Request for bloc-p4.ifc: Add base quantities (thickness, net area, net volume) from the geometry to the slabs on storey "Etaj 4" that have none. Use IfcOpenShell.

First a look at what the model holds.

```python
import ifcopenshell
import ifcopenshell.util.element
import ifcopenshell.util.unit

model = ifcopenshell.open("bloc-p4.ifc")
print(model.schema)
for unit_type in ("LENGTHUNIT", "AREAUNIT", "VOLUMEUNIT"):
    print(unit_type, ifcopenshell.util.unit.calculate_unit_scale(model, unit_type))
storey = next(s for s in model.by_type("IfcBuildingStorey") if s.Name == "Etaj 4")
slabs = [e for e in ifcopenshell.util.element.get_decomposition(storey) if e.is_a("IfcSlab")]
for e in sorted(slabs, key=lambda e: e.id()):
    print(e.id(), e.is_a(), e.Name, list(ifcopenshell.util.element.get_psets(e, qtos_only=True)), sep=" | ")
```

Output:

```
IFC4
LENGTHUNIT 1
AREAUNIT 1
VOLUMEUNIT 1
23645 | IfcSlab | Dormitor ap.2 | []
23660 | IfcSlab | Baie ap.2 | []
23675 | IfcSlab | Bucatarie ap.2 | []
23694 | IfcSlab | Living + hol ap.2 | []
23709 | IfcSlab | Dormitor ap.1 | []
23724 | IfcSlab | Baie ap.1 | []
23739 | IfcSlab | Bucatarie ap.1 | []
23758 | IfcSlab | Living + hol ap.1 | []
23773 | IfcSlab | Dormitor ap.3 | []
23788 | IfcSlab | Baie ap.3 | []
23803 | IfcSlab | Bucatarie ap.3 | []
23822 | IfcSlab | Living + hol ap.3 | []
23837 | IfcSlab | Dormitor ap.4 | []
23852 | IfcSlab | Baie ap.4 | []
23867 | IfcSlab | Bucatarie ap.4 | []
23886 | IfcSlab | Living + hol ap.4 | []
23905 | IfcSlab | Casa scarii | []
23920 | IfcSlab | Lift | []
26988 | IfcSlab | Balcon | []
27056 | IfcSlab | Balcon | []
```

```python
import ifcopenshell
import ifcopenshell.api.pset
import ifcopenshell.geom
import ifcopenshell.util.element
import ifcopenshell.util.shape
import ifcopenshell.util.unit

model = ifcopenshell.open("bloc-p4.ifc")
unit_scale = ifcopenshell.util.unit.calculate_unit_scale(model)
area_scale = ifcopenshell.util.unit.calculate_unit_scale(model, "AREAUNIT")
volume_scale = ifcopenshell.util.unit.calculate_unit_scale(model, "VOLUMEUNIT")
settings = ifcopenshell.geom.settings()

storey = next(s for s in model.by_type("IfcBuildingStorey") if s.Name == "Etaj 4")
slabs = [e for e in ifcopenshell.util.element.get_decomposition(storey) if e.is_a("IfcSlab")]

for e in sorted(slabs, key=lambda e: e.id()):
    if ifcopenshell.util.element.get_psets(e, qtos_only=True, should_inherit=False):
        continue
    # Geometry comes back in metres, in the element's own axes.
    shape = ifcopenshell.geom.create_shape(settings, e)
    values = {
        "Width": ifcopenshell.util.shape.get_z(shape.geometry) / unit_scale,
        "NetArea": ifcopenshell.util.shape.get_footprint_area(shape.geometry) / area_scale,
        "NetVolume": ifcopenshell.util.shape.get_volume(shape.geometry) / volume_scale,
    }
    qto = ifcopenshell.api.pset.add_qto(model, product=e, name="Qto_SlabBaseQuantities")
    ifcopenshell.api.pset.edit_qto(model, qto=qto, properties=values)
    print(e.id(), {k: round(v, 3) for k, v in values.items()})

model.write("bloc-p4_rev.ifc")
```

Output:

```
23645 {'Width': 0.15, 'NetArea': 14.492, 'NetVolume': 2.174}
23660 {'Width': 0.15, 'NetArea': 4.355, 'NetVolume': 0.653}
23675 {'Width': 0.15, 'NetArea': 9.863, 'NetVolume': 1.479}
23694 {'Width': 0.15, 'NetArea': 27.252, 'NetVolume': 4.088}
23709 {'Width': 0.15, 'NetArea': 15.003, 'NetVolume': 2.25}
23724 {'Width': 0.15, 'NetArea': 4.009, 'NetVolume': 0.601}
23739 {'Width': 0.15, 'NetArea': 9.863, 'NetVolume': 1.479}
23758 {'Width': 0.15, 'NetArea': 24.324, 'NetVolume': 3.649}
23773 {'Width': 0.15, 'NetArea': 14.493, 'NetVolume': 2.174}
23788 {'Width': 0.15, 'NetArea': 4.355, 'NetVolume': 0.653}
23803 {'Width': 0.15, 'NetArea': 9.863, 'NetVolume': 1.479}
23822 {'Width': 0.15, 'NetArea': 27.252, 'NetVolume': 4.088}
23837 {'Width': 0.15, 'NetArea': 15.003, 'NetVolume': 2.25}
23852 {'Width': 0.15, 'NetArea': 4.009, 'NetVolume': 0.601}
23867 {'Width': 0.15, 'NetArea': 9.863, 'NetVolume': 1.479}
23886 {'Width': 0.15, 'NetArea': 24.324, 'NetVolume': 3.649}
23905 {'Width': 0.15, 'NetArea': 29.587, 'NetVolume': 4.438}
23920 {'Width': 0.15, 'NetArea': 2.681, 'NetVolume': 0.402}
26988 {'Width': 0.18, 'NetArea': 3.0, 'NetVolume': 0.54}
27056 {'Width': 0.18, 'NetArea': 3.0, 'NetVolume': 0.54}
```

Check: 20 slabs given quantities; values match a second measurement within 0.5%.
